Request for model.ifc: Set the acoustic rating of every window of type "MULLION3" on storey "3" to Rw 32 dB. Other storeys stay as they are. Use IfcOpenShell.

First a look at what the model holds.

```python
import ifcopenshell
import ifcopenshell.util.element

model = ifcopenshell.open("model.ifc")
print(model.schema)
storey = next(s for s in model.by_type("IfcBuildingStorey") if s.Name == "3")
windows = [e for e in ifcopenshell.util.element.get_decomposition(storey) if e.is_a("IfcWindow")]
seen = {}
for e in windows:
    element_type = ifcopenshell.util.element.get_type(e)
    key = (element_type.Name if element_type != e and element_type else None, ifcopenshell.util.element.get_pset(e, "Pset_WindowCommon", "AcousticRating"))
    seen[key] = seen.get(key, 0) + 1
for (name, value), count in sorted(seen.items(), key=str):
    print(count, "x", name, "|", value)
```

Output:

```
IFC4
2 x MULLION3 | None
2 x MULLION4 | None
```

```python
import ifcopenshell
import ifcopenshell.api.pset
import ifcopenshell.util.element

model = ifcopenshell.open("model.ifc")

storey = next(s for s in model.by_type("IfcBuildingStorey") if s.Name == "3")
windows = [e for e in ifcopenshell.util.element.get_decomposition(storey) if e.is_a("IfcWindow")]

count = 0
for e in windows:
    element_type = ifcopenshell.util.element.get_type(e)
    if element_type in (None, e) or element_type.Name != "MULLION3":
        continue
    # add_pset returns the element's existing set when there is one.
    pset = ifcopenshell.api.pset.add_pset(model, product=e, name="Pset_WindowCommon")
    ifcopenshell.api.pset.edit_pset(model, pset=pset, properties={"AcousticRating": "Rw 32 dB"})
    count += 1

print(count, "windows updated")

model.write("model_edited.ifc")
```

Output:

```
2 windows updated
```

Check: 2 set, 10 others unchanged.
